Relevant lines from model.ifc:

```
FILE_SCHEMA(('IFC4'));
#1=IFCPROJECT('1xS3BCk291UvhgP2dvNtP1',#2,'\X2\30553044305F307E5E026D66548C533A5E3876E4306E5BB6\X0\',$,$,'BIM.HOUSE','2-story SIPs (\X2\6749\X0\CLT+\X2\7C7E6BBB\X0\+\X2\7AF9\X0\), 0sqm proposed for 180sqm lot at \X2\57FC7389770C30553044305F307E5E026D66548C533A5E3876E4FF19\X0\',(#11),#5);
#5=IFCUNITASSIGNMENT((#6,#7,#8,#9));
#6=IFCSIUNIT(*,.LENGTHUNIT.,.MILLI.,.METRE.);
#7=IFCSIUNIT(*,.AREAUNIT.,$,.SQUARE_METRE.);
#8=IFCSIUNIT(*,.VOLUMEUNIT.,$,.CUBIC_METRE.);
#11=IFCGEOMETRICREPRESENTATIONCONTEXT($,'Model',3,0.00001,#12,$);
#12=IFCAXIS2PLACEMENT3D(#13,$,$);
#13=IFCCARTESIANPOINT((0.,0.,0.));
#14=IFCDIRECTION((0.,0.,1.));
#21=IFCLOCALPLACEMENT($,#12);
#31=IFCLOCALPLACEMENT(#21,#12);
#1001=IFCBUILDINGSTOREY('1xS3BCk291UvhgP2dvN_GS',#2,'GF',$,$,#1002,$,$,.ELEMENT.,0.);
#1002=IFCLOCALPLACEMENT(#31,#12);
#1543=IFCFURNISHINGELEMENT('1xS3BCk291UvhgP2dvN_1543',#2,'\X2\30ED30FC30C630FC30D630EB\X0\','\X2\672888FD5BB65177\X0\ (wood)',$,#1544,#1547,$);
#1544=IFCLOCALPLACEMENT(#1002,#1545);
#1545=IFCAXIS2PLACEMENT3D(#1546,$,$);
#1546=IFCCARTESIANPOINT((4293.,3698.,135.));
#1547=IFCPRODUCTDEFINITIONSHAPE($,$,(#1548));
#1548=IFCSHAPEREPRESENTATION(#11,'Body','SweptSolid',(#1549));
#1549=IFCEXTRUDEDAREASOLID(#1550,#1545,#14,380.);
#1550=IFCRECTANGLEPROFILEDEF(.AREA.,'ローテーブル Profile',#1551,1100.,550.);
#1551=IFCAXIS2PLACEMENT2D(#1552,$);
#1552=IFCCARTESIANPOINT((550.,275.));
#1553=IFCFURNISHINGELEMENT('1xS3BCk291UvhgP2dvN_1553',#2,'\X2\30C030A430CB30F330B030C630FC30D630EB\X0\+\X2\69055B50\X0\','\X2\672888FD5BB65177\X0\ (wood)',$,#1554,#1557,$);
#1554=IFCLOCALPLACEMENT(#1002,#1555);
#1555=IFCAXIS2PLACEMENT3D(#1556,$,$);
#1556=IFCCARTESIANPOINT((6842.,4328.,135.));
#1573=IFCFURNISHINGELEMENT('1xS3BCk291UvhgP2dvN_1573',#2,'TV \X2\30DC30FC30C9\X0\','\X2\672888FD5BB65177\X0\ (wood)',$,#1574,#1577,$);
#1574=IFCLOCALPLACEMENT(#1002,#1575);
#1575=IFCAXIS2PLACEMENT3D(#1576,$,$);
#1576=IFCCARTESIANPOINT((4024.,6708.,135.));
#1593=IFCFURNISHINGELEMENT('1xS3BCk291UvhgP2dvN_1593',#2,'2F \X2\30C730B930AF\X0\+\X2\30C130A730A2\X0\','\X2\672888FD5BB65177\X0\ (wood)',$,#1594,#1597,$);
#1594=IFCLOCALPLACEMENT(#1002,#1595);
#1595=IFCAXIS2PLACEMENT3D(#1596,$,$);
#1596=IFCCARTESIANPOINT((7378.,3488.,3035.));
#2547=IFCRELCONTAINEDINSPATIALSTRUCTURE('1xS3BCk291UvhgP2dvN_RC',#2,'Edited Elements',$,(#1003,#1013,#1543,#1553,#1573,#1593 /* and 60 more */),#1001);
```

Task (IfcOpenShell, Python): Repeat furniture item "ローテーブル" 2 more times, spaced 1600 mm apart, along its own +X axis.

```python
import ifcopenshell
import ifcopenshell.api.geometry
import ifcopenshell.api.root
import ifcopenshell.util.element
import ifcopenshell.util.placement
import ifcopenshell.util.unit

model = ifcopenshell.open("model.ifc")
unit_scale = ifcopenshell.util.unit.calculate_unit_scale(model)


def reuse_history(source, copy):
    """copy_class also copies each property set's owner history, people and application; keep the originals."""
    for rel in copy.IsDefinedBy:
        if rel.is_a("IfcRelDefinesByProperties") and (history := rel.RelatingPropertyDefinition.OwnerHistory):
            rel.RelatingPropertyDefinition.OwnerHistory = source.OwnerHistory
            ifcopenshell.util.element.remove_deep2(model, history)


source = model.by_id(1543)
base = ifcopenshell.util.placement.get_local_placement(source.ObjectPlacement)
step = base[:3, 0] * 1.6 / unit_scale

for i in range(1, 3):
    copy = ifcopenshell.api.root.copy_class(model, product=source)
    copy.Representation = ifcopenshell.util.element.copy_deep(
        model, source.Representation, exclude=["IfcGeometricRepresentationContext", "IfcRepresentationMap"]
    )
    reuse_history(source, copy)
    matrix = base.copy()
    matrix[:3, 3] += i * step
    print("added at", matrix[:3, 3].round(3) + 0.0)
    ifcopenshell.api.geometry.edit_object_placement(model, product=copy, matrix=matrix, is_si=False)

model.write("model_updated.ifc")
```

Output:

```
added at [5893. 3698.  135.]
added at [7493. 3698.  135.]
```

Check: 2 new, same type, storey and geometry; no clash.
